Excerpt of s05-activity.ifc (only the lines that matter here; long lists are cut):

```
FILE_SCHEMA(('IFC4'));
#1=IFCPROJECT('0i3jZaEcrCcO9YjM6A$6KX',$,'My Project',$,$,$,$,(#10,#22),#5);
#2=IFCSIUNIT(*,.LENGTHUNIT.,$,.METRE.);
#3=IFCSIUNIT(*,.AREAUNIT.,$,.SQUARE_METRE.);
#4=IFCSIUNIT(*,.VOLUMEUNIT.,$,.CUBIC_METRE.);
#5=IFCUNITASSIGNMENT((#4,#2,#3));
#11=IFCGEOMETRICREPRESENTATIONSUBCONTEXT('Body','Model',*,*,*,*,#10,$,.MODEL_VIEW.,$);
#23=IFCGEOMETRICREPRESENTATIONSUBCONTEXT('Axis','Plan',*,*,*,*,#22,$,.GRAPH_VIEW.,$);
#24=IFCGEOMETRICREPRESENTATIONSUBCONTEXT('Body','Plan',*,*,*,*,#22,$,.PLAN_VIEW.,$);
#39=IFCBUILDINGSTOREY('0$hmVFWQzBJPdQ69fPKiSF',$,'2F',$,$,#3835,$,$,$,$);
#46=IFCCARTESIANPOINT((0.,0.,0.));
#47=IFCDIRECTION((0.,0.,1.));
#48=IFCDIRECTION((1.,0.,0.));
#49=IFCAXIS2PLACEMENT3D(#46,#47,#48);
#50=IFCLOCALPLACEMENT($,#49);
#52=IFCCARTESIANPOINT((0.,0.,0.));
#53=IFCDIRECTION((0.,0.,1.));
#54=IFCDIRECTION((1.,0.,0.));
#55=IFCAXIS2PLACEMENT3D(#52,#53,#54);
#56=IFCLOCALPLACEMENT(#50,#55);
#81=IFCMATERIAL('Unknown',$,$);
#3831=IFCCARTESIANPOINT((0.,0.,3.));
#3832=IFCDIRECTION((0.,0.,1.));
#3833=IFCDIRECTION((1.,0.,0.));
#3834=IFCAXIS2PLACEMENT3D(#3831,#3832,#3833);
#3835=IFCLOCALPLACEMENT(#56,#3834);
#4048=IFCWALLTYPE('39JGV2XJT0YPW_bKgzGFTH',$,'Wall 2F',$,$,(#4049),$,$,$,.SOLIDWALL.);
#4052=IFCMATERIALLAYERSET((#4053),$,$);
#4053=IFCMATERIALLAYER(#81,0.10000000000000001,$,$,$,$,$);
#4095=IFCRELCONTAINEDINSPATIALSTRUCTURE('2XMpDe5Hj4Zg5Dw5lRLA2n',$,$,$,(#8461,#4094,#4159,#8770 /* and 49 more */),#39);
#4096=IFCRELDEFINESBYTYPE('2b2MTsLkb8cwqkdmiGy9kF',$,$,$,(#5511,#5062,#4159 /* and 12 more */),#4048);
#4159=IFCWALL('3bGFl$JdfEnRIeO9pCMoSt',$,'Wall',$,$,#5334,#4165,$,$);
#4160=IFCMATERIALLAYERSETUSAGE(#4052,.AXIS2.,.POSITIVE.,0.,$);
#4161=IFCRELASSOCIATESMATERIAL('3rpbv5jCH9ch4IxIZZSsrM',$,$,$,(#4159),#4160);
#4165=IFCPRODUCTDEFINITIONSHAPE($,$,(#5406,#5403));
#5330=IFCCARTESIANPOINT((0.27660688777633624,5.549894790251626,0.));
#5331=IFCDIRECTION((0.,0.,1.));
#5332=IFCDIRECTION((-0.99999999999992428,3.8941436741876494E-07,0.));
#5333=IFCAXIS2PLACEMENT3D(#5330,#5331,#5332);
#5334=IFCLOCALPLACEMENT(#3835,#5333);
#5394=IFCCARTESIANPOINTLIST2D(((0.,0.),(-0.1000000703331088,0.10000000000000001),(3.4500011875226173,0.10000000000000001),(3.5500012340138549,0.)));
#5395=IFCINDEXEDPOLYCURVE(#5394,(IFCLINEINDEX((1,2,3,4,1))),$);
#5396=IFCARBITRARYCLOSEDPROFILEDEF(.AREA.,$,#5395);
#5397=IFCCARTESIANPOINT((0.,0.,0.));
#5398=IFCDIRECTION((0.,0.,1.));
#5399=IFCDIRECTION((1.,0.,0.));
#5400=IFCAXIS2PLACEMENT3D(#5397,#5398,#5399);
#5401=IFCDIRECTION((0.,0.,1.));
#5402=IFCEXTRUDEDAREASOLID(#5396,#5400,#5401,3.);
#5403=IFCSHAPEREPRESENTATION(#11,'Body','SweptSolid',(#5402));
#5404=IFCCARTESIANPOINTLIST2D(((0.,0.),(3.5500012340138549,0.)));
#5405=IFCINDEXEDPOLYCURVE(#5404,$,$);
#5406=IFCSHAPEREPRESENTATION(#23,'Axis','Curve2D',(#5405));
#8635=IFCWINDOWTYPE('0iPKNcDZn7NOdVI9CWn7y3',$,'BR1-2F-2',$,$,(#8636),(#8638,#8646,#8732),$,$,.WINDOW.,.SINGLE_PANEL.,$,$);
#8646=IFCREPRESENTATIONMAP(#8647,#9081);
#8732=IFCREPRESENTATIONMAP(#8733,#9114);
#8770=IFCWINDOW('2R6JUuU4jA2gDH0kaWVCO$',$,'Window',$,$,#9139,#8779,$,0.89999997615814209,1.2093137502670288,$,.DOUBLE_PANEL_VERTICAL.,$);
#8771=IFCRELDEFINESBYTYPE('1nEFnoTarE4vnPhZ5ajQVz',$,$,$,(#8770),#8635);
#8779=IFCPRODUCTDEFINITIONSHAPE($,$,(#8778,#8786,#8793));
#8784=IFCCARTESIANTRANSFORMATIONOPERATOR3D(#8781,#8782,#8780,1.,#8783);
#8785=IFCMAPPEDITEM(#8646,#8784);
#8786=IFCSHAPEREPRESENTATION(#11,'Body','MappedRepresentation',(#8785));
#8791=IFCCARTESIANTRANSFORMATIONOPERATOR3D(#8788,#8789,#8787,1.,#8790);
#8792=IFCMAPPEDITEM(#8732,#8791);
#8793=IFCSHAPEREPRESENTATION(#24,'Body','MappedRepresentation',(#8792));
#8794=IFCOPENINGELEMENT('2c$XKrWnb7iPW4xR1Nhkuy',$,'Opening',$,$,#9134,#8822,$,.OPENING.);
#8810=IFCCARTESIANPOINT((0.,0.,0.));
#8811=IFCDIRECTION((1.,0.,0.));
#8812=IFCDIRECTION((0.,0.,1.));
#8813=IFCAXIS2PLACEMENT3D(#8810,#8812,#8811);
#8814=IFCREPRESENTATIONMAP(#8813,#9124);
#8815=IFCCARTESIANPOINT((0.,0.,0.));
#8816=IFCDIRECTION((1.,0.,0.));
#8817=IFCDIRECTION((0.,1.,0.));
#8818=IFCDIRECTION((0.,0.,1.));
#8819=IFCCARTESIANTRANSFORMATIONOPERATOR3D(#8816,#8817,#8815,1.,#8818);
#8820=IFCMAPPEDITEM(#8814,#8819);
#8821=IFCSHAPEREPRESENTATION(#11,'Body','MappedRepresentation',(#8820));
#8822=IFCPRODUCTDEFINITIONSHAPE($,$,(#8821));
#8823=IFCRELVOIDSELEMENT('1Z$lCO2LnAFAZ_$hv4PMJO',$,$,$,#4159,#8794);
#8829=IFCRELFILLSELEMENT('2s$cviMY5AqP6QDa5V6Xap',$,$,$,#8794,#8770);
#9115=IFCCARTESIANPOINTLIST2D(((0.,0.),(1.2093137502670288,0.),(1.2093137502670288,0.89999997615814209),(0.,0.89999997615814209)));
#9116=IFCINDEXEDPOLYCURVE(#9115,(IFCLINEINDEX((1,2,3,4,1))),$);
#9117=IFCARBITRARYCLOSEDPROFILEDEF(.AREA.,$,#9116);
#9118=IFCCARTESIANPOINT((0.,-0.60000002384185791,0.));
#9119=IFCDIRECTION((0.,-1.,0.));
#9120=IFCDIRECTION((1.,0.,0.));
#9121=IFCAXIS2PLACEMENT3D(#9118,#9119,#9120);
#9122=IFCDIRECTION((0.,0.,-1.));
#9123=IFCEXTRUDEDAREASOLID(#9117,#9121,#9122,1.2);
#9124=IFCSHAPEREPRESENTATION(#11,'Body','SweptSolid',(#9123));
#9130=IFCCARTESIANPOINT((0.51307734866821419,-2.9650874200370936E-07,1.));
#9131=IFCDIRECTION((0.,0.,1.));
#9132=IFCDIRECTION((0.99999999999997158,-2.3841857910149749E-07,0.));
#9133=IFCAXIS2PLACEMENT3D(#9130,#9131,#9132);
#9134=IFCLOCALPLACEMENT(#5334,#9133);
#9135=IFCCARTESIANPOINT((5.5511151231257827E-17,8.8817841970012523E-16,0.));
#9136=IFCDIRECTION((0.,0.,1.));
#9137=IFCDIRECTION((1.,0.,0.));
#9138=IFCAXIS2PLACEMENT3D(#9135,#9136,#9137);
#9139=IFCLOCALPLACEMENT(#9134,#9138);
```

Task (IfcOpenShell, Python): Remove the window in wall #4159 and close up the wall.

```python
import ifcopenshell
import ifcopenshell.api.feature
import ifcopenshell.api.root
import ifcopenshell.geom
import ifcopenshell.util.shape

model = ifcopenshell.open("s05-activity.ifc")
settings = ifcopenshell.geom.settings()


def volume(element):
    """Net volume in cubic metres, openings subtracted."""
    shape = ifcopenshell.geom.create_shape(settings, element)
    return ifcopenshell.util.shape.get_volume(shape.geometry)


window = model.by_guid("2R6JUuU4jA2gDH0kaWVCO$")
opening = window.FillsVoids[0].RelatingOpeningElement
wall = opening.VoidsElements[0].RelatingBuildingElement
before = volume(wall)

ifcopenshell.api.root.remove_product(model, product=window)
ifcopenshell.api.feature.remove_feature(model, feature=opening)

after = volume(wall)

print(f"wall volume {before:.3f} -> {after:.3f} m3")

model.write("s05-activity-out.ifc")
```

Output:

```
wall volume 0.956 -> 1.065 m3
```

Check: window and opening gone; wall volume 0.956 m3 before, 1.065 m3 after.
